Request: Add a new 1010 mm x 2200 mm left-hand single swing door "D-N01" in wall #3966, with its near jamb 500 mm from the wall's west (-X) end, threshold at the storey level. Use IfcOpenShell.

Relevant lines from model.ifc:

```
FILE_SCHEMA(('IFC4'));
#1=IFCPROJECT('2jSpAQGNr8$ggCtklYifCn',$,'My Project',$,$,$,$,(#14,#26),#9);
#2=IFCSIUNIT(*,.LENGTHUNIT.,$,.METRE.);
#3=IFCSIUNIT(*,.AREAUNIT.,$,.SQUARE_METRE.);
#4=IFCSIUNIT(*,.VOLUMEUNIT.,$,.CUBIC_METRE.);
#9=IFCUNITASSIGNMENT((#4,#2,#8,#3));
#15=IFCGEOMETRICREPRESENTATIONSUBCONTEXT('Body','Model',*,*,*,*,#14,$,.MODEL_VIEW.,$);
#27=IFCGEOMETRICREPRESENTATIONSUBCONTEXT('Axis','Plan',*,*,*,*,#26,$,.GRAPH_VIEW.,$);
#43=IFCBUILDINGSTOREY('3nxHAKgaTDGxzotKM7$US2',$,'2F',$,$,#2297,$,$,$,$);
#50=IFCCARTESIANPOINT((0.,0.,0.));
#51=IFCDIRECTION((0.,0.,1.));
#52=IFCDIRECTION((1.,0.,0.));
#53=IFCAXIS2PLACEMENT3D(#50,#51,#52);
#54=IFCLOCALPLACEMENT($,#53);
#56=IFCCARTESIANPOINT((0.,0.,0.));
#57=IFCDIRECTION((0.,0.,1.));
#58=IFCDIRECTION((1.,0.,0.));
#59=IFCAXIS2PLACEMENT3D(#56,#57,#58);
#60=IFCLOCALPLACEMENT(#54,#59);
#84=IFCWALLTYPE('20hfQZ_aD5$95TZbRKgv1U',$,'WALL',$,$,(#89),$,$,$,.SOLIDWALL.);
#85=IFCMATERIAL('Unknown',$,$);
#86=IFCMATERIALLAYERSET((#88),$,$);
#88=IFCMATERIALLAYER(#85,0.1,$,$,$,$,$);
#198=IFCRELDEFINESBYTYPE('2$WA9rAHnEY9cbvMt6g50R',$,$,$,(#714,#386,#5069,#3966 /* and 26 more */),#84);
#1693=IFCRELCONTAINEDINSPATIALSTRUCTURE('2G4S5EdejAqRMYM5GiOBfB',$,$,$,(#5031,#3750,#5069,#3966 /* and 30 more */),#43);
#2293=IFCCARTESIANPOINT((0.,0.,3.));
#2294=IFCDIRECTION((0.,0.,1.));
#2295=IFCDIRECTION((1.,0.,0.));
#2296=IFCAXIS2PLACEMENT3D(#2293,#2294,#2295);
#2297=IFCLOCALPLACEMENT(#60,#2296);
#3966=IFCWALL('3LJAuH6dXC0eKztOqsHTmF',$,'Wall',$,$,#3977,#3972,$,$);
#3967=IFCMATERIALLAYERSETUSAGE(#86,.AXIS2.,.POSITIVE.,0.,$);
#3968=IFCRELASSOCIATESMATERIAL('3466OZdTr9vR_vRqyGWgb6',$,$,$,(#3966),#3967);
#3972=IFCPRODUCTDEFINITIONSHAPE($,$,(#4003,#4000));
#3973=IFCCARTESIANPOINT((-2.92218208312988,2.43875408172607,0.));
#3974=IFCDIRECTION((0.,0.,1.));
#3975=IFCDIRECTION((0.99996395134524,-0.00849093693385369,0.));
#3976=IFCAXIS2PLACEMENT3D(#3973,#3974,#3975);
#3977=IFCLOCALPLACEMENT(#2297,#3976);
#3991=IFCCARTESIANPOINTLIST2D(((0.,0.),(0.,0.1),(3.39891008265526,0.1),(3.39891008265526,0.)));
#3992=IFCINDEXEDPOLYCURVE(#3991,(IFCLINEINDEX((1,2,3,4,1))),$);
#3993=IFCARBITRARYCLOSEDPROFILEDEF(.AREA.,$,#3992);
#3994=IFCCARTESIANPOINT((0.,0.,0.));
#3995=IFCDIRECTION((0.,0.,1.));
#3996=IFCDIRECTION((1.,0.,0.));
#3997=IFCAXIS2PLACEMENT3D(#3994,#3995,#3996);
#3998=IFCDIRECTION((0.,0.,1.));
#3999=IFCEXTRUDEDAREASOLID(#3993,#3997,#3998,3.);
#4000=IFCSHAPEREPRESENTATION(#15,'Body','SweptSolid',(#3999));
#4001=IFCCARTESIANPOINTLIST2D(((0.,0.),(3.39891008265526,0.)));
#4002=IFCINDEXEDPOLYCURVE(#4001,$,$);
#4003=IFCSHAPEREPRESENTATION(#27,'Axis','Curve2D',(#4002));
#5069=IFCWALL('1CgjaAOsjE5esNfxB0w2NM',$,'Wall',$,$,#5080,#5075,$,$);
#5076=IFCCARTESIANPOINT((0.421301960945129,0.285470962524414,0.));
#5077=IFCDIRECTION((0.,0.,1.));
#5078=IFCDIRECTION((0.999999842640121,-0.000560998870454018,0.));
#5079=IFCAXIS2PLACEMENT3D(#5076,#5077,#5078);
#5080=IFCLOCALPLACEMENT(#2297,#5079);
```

```python
import numpy as np
import ifcopenshell
import ifcopenshell.api.feature
import ifcopenshell.api.geometry
import ifcopenshell.api.root
import ifcopenshell.api.spatial
import ifcopenshell.geom
import ifcopenshell.util.element
import ifcopenshell.util.placement
import ifcopenshell.util.representation
import ifcopenshell.util.shape
import ifcopenshell.util.unit

model = ifcopenshell.open("model.ifc")
unit_scale = ifcopenshell.util.unit.calculate_unit_scale(model)
settings = ifcopenshell.geom.settings()


def volume(element):
    """Net volume in cubic metres, openings subtracted."""
    shape = ifcopenshell.geom.create_shape(settings, element)
    return ifcopenshell.util.shape.get_volume(shape.geometry)


wall = model.by_id(3966)
storey = ifcopenshell.util.element.get_container(wall, ifc_class="IfcBuildingStorey")
context = ifcopenshell.util.representation.get_context(model, "Model", "Body", "MODEL_VIEW")
before = volume(wall)

width, height, from_end, sill = 1.01, 2.2, 0.5, 0.0  # metres

# The wall runs along its own X axis, and the end named is its -X end.
wall_shape = ifcopenshell.geom.create_shape(settings, wall)
x, y, z = ifcopenshell.util.shape.get_vertices(wall_shape.geometry).T
start = x.min() + from_end
face, thickness = float(y.min()), float(y.max() - y.min())
wall_matrix = ifcopenshell.util.placement.get_local_placement(wall.ObjectPlacement)
level = ifcopenshell.util.placement.get_local_placement(storey.ObjectPlacement)[2, 3]


def in_wall(x, y):
    """Placement at x, y metres in the wall's axes, at sill height."""
    matrix = wall_matrix.copy()
    matrix[:, 3] = wall_matrix @ np.array([x / unit_scale, y / unit_scale, 0.0, 1.0])
    matrix[2, 3] = level + sill / unit_scale
    return matrix


# Opening: a box that overshoots both wall faces by 50 mm.
opening = ifcopenshell.api.root.create_entity(model, ifc_class="IfcOpeningElement", predefined_type="OPENING")
box = ifcopenshell.api.geometry.add_wall_representation(
    model, context=context, length=width, height=height, thickness=thickness + 0.1
)
ifcopenshell.api.geometry.assign_representation(model, product=opening, representation=box)
ifcopenshell.api.geometry.edit_object_placement(model, product=opening, matrix=in_wall(start, face - 0.05), is_si=False)
ifcopenshell.api.feature.add_feature(model, feature=opening, element=wall)

door = ifcopenshell.api.root.create_entity(model, ifc_class="IfcDoor", name="D-N01", predefined_type="DOOR")
door.OverallWidth, door.OverallHeight = width / unit_scale, height / unit_scale
door.OperationType = "SINGLE_SWING_LEFT"
body = ifcopenshell.api.geometry.add_door_representation(
    model,
    context=context,
    overall_width=door.OverallWidth,
    overall_height=door.OverallHeight,
    operation_type="SINGLE_SWING_LEFT",
    lining_properties={"LiningDepth": thickness / unit_scale, "ThresholdDepth": thickness / unit_scale},
)
ifcopenshell.api.geometry.assign_representation(model, product=door, representation=body)
ifcopenshell.api.spatial.assign_container(model, products=[door], relating_structure=storey)
ifcopenshell.api.feature.add_filling(model, opening=opening, element=door)

# The lining spans the wall, so the door starts at the wall face.
ifcopenshell.api.geometry.edit_object_placement(model, product=door, matrix=in_wall(start, face), is_si=False)

after = volume(wall)

print(f"wall volume {before:.3f} -> {after:.3f} m3")

model.write("model_updated.ifc")
```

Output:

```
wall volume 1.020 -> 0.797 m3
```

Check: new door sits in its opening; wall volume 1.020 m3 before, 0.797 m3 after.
